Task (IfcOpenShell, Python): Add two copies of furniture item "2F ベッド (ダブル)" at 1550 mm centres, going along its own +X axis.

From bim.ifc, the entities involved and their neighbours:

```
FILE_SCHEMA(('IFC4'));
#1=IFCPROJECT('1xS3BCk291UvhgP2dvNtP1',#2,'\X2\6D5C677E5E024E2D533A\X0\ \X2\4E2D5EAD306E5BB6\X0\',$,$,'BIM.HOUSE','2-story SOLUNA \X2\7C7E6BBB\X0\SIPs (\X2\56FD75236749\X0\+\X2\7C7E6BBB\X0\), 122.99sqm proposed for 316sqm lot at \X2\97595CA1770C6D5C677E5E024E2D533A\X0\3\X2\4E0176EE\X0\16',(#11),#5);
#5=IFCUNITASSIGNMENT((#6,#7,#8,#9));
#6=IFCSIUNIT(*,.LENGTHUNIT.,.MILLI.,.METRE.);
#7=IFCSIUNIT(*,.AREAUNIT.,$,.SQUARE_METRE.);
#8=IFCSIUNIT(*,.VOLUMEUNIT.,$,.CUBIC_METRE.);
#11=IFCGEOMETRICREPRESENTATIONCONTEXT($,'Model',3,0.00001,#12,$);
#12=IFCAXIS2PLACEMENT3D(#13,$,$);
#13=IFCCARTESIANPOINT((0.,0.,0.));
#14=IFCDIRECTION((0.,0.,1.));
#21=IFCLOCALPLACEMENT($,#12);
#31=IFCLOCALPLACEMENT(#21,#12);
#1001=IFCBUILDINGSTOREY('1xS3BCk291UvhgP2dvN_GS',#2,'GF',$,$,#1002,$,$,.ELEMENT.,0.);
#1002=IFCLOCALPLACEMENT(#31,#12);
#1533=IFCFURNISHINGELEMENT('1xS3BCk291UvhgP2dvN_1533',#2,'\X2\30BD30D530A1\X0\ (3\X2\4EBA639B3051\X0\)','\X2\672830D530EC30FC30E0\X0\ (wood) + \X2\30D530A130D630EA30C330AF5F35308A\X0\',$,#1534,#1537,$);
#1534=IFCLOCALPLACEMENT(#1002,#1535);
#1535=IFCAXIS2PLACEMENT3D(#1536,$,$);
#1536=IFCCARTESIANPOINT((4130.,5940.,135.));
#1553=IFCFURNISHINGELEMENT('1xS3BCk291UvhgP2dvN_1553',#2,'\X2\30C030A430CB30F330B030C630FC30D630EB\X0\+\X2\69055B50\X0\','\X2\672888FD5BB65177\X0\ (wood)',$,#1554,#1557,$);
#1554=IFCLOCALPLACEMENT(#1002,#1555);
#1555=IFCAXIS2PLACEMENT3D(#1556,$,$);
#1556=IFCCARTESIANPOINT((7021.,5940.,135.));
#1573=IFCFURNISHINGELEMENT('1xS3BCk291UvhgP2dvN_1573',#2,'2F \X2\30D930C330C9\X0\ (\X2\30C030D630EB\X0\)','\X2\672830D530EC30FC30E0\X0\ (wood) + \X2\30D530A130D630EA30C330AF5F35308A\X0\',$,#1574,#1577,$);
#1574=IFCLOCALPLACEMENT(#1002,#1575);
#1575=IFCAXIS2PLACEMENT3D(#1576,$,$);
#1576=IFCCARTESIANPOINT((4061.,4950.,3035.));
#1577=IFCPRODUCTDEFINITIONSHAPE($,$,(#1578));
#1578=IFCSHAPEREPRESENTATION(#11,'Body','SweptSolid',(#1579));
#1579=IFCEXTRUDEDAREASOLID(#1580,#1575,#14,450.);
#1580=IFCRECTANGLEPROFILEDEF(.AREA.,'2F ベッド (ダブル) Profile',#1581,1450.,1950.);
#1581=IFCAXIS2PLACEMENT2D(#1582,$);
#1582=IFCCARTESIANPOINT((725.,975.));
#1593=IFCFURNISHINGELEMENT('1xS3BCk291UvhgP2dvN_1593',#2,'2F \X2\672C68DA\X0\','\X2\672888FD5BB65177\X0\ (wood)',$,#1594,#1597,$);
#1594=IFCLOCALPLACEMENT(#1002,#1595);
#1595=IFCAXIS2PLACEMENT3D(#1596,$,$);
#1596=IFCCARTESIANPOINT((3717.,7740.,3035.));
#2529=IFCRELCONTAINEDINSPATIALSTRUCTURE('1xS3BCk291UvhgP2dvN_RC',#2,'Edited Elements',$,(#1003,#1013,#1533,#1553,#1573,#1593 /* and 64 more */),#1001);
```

```python
import ifcopenshell
import ifcopenshell.api.geometry
import ifcopenshell.api.root
import ifcopenshell.util.element
import ifcopenshell.util.placement
import ifcopenshell.util.unit

model = ifcopenshell.open("bim.ifc")
unit_scale = ifcopenshell.util.unit.calculate_unit_scale(model)


def reuse_history(source, copy):
    """copy_class also copies each property set's owner history, people and application; keep the originals."""
    for rel in copy.IsDefinedBy:
        if rel.is_a("IfcRelDefinesByProperties") and (history := rel.RelatingPropertyDefinition.OwnerHistory):
            rel.RelatingPropertyDefinition.OwnerHistory = source.OwnerHistory
            ifcopenshell.util.element.remove_deep2(model, history)


source = model.by_guid("1xS3BCk291UvhgP2dvN_1573")
base = ifcopenshell.util.placement.get_local_placement(source.ObjectPlacement)
step = base[:3, 0] * 1.55 / unit_scale

for i in range(1, 3):
    copy = ifcopenshell.api.root.copy_class(model, product=source)
    copy.Representation = ifcopenshell.util.element.copy_deep(
        model, source.Representation, exclude=["IfcGeometricRepresentationContext", "IfcRepresentationMap"]
    )
    reuse_history(source, copy)
    matrix = base.copy()
    matrix[:3, 3] += i * step
    print("added at", matrix[:3, 3].round(3) + 0.0)
    ifcopenshell.api.geometry.edit_object_placement(model, product=copy, matrix=matrix, is_si=False)

model.write("bim_rev.ifc")
```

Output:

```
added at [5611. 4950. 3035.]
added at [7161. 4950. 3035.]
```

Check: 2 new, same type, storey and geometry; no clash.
